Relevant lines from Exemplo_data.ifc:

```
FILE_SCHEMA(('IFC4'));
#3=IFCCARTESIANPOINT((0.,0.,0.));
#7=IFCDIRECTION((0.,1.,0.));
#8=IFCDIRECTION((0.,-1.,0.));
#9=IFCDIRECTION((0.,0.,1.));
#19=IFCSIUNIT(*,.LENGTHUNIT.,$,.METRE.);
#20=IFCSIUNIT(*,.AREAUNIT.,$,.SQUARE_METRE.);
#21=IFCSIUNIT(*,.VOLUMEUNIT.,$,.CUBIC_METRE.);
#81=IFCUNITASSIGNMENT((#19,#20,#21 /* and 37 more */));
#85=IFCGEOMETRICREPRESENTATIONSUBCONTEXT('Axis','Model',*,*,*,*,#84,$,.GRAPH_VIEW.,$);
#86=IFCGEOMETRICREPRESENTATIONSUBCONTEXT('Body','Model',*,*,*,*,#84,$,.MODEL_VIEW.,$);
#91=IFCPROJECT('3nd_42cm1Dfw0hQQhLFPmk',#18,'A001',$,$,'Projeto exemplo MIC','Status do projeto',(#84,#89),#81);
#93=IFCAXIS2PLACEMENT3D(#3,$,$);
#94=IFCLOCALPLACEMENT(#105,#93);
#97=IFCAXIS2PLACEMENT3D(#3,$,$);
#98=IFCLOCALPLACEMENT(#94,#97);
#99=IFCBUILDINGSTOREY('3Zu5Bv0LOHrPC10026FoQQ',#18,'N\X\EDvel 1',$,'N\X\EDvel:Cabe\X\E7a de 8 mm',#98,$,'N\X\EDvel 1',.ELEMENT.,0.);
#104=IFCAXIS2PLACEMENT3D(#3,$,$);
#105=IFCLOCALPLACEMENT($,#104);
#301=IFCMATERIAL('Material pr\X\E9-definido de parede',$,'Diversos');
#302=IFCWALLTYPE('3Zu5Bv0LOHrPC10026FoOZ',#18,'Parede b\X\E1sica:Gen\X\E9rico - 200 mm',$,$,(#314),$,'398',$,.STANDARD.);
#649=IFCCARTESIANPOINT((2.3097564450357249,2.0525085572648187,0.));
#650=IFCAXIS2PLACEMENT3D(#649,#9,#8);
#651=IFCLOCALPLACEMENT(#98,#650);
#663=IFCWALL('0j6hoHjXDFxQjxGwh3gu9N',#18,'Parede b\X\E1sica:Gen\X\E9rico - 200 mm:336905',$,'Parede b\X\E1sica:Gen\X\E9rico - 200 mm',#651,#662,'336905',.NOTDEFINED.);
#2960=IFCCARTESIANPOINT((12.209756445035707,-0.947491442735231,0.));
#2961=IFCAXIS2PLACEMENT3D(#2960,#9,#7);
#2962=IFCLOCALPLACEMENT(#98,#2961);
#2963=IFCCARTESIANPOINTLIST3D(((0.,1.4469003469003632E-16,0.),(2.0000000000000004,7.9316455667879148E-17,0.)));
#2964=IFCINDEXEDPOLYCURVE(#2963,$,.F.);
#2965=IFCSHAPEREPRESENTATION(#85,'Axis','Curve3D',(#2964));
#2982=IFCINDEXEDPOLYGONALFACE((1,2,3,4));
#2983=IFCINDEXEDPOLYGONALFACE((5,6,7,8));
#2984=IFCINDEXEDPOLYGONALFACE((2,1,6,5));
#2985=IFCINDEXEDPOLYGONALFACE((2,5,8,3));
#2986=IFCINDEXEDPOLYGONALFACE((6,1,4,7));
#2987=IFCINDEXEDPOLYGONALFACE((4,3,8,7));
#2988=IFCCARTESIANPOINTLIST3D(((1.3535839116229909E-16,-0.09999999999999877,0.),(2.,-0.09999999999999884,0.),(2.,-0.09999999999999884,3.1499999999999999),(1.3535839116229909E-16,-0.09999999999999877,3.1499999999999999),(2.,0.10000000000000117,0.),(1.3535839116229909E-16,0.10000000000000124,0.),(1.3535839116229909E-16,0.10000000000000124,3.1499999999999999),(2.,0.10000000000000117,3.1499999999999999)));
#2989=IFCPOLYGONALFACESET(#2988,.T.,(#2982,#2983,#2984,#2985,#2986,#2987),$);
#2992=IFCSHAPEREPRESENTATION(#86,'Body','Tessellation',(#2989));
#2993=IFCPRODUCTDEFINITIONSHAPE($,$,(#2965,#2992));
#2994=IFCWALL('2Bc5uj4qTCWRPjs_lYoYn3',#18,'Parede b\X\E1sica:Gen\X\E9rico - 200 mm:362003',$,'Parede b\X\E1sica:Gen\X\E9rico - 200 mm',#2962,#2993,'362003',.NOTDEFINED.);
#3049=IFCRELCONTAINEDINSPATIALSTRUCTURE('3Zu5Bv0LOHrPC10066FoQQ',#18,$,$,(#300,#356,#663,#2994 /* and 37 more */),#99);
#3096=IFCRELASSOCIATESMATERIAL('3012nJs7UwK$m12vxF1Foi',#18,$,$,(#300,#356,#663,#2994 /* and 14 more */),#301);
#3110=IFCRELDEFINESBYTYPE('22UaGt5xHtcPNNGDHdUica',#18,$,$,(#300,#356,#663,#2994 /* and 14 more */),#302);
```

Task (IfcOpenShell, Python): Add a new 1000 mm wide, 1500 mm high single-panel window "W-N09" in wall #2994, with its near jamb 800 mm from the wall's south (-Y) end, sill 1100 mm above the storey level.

```python
import numpy as np
import ifcopenshell
import ifcopenshell.api.feature
import ifcopenshell.api.geometry
import ifcopenshell.api.root
import ifcopenshell.api.spatial
import ifcopenshell.geom
import ifcopenshell.util.element
import ifcopenshell.util.placement
import ifcopenshell.util.representation
import ifcopenshell.util.shape
import ifcopenshell.util.unit

model = ifcopenshell.open("Exemplo_data.ifc")
unit_scale = ifcopenshell.util.unit.calculate_unit_scale(model)
settings = ifcopenshell.geom.settings()


def volume(element):
    """Net volume in cubic metres, openings subtracted."""
    shape = ifcopenshell.geom.create_shape(settings, element)
    return ifcopenshell.util.shape.get_volume(shape.geometry)


wall = model.by_id(2994)
storey = ifcopenshell.util.element.get_container(wall, ifc_class="IfcBuildingStorey")
context = ifcopenshell.util.representation.get_context(model, "Model", "Body", "MODEL_VIEW")
before = volume(wall)

width, height, from_end, sill = 1, 1.5, 0.8, 1.1  # metres

# The wall runs along its own X axis, and the end named is its -X end.
wall_shape = ifcopenshell.geom.create_shape(settings, wall)
x, y, z = ifcopenshell.util.shape.get_vertices(wall_shape.geometry).T
start = x.min() + from_end
face, thickness = float(y.min()), float(y.max() - y.min())
wall_matrix = ifcopenshell.util.placement.get_local_placement(wall.ObjectPlacement)
level = ifcopenshell.util.placement.get_local_placement(storey.ObjectPlacement)[2, 3]


def in_wall(x, y):
    """Placement at x, y metres in the wall's axes, at sill height."""
    matrix = wall_matrix.copy()
    matrix[:, 3] = wall_matrix @ np.array([x / unit_scale, y / unit_scale, 0.0, 1.0])
    matrix[2, 3] = level + sill / unit_scale
    return matrix


# Opening: a box that overshoots both wall faces by 50 mm.
opening = ifcopenshell.api.root.create_entity(model, ifc_class="IfcOpeningElement", predefined_type="OPENING")
box = ifcopenshell.api.geometry.add_wall_representation(
    model, context=context, length=width, height=height, thickness=thickness + 0.1
)
ifcopenshell.api.geometry.assign_representation(model, product=opening, representation=box)
ifcopenshell.api.geometry.edit_object_placement(model, product=opening, matrix=in_wall(start, face - 0.05), is_si=False)
ifcopenshell.api.feature.add_feature(model, feature=opening, element=wall)

window = ifcopenshell.api.root.create_entity(model, ifc_class="IfcWindow", name="W-N09", predefined_type="WINDOW")
window.OverallWidth, window.OverallHeight = width / unit_scale, height / unit_scale
window.PartitioningType = "SINGLE_PANEL"
body = ifcopenshell.api.geometry.add_window_representation(
    model,
    context=context,
    overall_width=window.OverallWidth,
    overall_height=window.OverallHeight,
    partition_type="SINGLE_PANEL",
)
ifcopenshell.api.geometry.assign_representation(model, product=window, representation=body)
ifcopenshell.api.spatial.assign_container(model, products=[window], relating_structure=storey)
ifcopenshell.api.feature.add_filling(model, opening=opening, element=window)

# Centre the window in the wall's thickness.
ifcopenshell.api.geometry.edit_object_placement(model, product=window, matrix=in_wall(start, face), is_si=False)
window_shape = ifcopenshell.geom.create_shape(settings, window)
depth = ifcopenshell.util.shape.get_vertices(window_shape.geometry)[:, 1]
offset = face + thickness / 2 - (depth.min() + depth.max()) / 2
ifcopenshell.api.geometry.edit_object_placement(model, product=window, matrix=in_wall(start, offset), is_si=False)

after = volume(wall)

print(f"wall volume {before:.3f} -> {after:.3f} m3")

model.write("Exemplo_data_rev.ifc")
```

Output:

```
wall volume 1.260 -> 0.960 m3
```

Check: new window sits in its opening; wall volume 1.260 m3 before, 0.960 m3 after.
